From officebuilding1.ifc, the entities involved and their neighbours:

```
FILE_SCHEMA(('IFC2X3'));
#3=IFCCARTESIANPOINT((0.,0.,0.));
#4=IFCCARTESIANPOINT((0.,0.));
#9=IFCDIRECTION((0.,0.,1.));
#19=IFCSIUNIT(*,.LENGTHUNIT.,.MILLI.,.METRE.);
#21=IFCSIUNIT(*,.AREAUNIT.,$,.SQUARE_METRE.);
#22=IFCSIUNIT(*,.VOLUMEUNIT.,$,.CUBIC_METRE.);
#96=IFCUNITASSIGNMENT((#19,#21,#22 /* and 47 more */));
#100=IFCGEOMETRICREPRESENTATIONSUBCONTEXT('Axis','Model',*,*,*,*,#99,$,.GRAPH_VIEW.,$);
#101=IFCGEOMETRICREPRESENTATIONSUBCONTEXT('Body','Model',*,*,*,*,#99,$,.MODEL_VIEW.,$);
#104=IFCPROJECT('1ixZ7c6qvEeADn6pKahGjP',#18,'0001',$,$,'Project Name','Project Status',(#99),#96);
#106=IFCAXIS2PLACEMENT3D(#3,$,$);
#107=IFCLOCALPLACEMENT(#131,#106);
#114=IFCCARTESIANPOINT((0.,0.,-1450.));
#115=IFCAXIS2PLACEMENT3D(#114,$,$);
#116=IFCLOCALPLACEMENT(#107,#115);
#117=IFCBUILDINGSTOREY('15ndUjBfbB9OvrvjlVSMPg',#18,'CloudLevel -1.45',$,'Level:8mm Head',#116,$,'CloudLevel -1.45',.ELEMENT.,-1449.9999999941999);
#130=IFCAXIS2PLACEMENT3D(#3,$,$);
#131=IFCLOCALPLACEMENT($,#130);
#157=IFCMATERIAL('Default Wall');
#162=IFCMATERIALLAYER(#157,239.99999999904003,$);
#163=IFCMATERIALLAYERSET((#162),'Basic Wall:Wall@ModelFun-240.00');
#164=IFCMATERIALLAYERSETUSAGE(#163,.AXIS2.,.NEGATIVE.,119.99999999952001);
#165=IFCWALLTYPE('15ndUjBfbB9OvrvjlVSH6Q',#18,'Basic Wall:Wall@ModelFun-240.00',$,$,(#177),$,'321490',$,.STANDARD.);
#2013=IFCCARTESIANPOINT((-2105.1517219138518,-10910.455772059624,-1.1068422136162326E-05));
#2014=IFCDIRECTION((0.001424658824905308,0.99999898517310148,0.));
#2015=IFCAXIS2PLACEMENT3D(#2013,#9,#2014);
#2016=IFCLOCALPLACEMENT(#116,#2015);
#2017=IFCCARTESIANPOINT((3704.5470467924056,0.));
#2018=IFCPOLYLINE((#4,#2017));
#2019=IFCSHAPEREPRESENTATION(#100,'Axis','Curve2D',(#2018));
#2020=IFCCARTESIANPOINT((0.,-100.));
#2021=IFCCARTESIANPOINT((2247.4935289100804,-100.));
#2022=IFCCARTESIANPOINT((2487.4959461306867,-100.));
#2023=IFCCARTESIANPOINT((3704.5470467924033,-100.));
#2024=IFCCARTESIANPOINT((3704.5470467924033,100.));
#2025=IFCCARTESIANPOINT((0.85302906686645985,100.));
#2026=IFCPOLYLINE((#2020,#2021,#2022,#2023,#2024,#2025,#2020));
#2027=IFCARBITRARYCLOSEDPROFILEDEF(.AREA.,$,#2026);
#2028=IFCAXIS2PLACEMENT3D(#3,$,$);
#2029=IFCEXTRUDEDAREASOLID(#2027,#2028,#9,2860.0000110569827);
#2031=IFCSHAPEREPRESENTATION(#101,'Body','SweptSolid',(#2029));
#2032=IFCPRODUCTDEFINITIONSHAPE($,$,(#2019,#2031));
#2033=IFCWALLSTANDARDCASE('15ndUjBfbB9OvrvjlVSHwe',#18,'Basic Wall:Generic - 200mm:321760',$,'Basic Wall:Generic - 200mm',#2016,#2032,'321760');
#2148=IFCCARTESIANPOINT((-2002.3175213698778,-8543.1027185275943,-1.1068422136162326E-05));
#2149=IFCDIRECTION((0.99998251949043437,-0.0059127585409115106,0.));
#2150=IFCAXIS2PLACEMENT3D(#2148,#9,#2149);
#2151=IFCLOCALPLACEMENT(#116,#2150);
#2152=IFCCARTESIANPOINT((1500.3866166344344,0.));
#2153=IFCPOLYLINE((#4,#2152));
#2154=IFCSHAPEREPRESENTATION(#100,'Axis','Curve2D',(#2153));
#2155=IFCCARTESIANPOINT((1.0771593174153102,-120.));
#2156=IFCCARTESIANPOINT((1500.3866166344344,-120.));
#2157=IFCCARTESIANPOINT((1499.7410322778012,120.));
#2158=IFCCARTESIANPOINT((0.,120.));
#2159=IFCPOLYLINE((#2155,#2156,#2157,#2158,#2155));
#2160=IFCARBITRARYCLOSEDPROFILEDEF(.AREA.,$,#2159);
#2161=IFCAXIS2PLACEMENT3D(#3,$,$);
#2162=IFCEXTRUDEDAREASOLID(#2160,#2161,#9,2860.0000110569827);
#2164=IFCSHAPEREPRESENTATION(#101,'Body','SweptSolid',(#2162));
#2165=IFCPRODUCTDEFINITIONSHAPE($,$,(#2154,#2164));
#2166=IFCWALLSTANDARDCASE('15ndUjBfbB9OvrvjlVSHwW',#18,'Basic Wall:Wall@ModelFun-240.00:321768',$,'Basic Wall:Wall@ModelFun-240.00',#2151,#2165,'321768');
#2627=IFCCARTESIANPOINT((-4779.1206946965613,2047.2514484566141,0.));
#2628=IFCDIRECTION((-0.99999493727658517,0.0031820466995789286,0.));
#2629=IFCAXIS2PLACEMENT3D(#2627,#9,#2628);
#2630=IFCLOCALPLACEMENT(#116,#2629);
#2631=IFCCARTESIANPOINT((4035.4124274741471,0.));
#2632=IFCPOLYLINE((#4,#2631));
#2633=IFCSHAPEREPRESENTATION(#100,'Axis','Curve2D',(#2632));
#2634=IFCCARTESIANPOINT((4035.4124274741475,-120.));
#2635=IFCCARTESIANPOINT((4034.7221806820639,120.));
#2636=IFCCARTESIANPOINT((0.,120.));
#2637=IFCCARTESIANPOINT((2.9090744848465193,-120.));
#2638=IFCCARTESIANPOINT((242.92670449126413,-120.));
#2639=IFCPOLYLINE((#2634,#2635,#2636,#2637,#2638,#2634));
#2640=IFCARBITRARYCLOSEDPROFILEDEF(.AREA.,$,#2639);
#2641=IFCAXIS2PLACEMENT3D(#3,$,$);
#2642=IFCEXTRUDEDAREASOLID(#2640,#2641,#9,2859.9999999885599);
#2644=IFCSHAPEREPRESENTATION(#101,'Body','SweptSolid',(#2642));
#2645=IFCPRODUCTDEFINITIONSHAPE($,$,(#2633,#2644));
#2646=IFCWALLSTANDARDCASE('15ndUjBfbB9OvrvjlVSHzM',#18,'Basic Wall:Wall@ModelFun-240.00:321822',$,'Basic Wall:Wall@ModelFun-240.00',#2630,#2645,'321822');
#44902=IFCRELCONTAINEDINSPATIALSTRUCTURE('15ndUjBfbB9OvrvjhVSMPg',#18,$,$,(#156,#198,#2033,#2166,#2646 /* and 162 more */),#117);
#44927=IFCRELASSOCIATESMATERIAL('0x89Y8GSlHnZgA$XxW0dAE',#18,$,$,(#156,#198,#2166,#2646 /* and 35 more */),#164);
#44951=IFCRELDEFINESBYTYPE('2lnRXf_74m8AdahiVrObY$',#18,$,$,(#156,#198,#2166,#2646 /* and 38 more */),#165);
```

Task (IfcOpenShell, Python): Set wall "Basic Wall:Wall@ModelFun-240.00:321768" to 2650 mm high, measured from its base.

```python
import ifcopenshell
import ifcopenshell.geom
import ifcopenshell.util.representation
import ifcopenshell.util.shape
import ifcopenshell.util.unit

model = ifcopenshell.open("officebuilding1.ifc")
unit_scale = ifcopenshell.util.unit.calculate_unit_scale(model)
settings = ifcopenshell.geom.settings()


def volume(element):
    """Net volume in cubic metres, openings subtracted."""
    shape = ifcopenshell.geom.create_shape(settings, element)
    return ifcopenshell.util.shape.get_volume(shape.geometry)


wall = model.by_guid("15ndUjBfbB9OvrvjlVSHwW")
before = volume(wall)

body = ifcopenshell.util.representation.get_representation(wall, "Model", "Body")
solid = body.Items[0]
old_height = solid.Depth
solid.Depth = 2.65 / unit_scale
after = volume(wall)

print(f"height {old_height:g} -> {solid.Depth:g}, volume {before:.3f} -> {after:.3f} m3")

model.write("officebuilding1-out.ifc")
```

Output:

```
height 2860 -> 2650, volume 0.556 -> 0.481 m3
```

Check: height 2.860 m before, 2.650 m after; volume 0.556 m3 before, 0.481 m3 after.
